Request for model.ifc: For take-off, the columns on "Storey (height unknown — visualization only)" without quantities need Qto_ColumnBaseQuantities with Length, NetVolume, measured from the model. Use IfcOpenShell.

First a look at what the model holds.

```python
import ifcopenshell
import ifcopenshell.util.element
import ifcopenshell.util.unit

model = ifcopenshell.open("model.ifc")
print(model.schema)
for unit_type in ("LENGTHUNIT", "AREAUNIT", "VOLUMEUNIT"):
    print(unit_type, ifcopenshell.util.unit.calculate_unit_scale(model, unit_type))
storey = next(s for s in model.by_type("IfcBuildingStorey") if s.Name == "Storey (height unknown — visualization only)")
columns = [e for e in ifcopenshell.util.element.get_decomposition(storey) if e.is_a("IfcColumn")]
for e in sorted(columns, key=lambda e: e.id()):
    print(e.id(), e.is_a(), e.Name, list(ifcopenshell.util.element.get_psets(e, qtos_only=True)), sep=" | ")
```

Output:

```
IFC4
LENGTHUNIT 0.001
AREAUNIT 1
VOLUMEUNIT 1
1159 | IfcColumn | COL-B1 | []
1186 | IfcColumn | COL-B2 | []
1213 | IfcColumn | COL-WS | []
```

```python
import ifcopenshell
import ifcopenshell.api.pset
import ifcopenshell.geom
import ifcopenshell.util.element
import ifcopenshell.util.shape
import ifcopenshell.util.unit

model = ifcopenshell.open("model.ifc")
unit_scale = ifcopenshell.util.unit.calculate_unit_scale(model)
volume_scale = ifcopenshell.util.unit.calculate_unit_scale(model, "VOLUMEUNIT")
settings = ifcopenshell.geom.settings()

storey = next(s for s in model.by_type("IfcBuildingStorey") if s.Name == "Storey (height unknown — visualization only)")
columns = [e for e in ifcopenshell.util.element.get_decomposition(storey) if e.is_a("IfcColumn")]

for e in sorted(columns, key=lambda e: e.id()):
    if ifcopenshell.util.element.get_psets(e, qtos_only=True, should_inherit=False):
        continue
    # Geometry comes back in metres, in the element's own axes.
    shape = ifcopenshell.geom.create_shape(settings, e)
    values = {
        "Length": ifcopenshell.util.shape.get_z(shape.geometry) / unit_scale,
        "NetVolume": ifcopenshell.util.shape.get_volume(shape.geometry) / volume_scale,
    }
    qto = ifcopenshell.api.pset.add_qto(model, product=e, name="Qto_ColumnBaseQuantities")
    ifcopenshell.api.pset.edit_qto(model, qto=qto, properties=values)
    print(e.id(), {k: round(v, 3) for k, v in values.items()})

model.write("model_edited.ifc")
```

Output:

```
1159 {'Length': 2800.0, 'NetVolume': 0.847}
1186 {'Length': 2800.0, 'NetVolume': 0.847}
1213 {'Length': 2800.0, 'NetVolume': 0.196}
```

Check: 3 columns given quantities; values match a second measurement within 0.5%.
